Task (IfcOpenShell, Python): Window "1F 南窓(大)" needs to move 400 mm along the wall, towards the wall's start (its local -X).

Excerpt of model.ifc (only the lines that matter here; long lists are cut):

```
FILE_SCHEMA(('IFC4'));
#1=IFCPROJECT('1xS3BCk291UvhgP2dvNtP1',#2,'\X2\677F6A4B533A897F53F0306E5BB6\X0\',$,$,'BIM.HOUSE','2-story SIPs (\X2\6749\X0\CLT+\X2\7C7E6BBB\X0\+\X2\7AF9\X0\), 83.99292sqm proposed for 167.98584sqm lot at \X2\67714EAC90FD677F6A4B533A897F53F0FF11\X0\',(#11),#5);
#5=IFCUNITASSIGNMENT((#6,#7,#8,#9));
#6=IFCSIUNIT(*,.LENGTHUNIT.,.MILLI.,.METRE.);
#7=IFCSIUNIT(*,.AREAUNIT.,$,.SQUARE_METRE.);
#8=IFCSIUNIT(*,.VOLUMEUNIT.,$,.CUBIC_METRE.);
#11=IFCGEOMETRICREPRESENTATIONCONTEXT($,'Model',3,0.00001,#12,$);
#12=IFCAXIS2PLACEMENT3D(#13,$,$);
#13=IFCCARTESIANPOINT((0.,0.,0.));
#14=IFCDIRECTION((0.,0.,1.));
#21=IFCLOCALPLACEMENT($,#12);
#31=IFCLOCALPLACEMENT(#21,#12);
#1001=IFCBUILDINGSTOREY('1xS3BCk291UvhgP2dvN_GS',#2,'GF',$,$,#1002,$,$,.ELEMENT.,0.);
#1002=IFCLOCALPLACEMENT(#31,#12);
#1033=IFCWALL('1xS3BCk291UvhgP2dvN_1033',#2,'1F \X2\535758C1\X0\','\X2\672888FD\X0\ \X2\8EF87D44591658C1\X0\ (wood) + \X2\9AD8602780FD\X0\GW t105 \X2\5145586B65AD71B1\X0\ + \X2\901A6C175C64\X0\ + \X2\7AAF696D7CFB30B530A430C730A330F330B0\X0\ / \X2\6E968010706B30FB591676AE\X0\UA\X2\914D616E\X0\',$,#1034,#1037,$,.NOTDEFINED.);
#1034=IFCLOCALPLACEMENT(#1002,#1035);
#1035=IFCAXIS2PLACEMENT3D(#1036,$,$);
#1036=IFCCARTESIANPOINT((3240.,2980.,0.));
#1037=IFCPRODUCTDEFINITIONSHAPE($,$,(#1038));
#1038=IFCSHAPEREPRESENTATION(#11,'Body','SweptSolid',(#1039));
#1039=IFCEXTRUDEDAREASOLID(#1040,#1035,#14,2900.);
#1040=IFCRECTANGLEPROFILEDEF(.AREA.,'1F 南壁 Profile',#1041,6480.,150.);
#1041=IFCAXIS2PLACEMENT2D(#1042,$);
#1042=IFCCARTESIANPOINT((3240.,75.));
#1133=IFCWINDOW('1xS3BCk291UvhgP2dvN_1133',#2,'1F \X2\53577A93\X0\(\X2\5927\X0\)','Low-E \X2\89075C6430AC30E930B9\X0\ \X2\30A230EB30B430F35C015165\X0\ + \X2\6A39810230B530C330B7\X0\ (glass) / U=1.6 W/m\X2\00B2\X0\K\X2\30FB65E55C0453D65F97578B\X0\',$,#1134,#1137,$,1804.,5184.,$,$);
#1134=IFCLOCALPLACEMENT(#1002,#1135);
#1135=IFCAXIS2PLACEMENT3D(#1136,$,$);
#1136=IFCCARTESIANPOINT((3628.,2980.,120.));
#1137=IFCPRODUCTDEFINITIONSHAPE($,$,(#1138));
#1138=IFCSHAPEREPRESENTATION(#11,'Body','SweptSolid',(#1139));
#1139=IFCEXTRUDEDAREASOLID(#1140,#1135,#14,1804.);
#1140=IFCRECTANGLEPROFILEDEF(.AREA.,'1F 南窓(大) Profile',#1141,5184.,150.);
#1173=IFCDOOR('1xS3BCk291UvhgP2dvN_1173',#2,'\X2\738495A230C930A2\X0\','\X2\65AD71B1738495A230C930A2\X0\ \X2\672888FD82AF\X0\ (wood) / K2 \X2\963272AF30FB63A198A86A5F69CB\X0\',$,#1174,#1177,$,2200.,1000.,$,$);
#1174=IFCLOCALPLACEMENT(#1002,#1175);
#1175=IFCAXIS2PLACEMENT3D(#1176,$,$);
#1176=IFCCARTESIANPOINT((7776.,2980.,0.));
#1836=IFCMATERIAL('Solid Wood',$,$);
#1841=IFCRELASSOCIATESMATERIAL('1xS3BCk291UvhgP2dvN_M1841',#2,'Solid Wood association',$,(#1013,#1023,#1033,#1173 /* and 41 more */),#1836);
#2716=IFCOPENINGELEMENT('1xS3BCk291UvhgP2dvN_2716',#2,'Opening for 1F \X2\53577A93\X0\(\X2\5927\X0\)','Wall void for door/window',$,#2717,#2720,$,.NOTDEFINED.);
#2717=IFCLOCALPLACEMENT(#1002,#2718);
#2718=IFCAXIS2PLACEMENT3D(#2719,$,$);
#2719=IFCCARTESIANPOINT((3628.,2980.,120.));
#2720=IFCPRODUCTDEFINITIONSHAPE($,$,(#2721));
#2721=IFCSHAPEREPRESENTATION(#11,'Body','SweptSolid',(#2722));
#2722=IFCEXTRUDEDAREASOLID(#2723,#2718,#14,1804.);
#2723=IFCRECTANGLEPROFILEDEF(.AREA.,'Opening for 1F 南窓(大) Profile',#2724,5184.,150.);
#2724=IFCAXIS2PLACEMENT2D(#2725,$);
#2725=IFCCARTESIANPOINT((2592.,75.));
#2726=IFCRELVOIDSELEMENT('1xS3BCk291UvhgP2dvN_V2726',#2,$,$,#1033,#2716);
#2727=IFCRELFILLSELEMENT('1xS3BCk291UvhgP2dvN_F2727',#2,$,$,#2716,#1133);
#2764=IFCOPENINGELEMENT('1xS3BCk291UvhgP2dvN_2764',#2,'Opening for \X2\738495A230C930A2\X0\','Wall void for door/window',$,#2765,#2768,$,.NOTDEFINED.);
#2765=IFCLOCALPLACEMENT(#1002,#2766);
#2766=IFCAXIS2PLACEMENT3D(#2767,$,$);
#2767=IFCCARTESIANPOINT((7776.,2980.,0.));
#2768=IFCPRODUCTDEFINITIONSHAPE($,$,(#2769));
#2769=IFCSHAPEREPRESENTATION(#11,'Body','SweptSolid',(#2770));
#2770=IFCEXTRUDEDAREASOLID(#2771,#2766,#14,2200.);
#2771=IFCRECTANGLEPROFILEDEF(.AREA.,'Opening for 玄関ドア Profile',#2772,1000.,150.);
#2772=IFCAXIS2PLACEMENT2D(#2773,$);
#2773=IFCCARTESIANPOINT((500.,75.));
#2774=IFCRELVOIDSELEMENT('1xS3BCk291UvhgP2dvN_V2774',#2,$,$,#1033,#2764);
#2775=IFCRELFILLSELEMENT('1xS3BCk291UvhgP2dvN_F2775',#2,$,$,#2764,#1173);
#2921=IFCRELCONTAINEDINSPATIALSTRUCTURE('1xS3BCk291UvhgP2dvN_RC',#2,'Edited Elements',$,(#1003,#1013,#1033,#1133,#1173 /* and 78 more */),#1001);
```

```python
import ifcopenshell
import ifcopenshell.api.geometry
import ifcopenshell.util.placement
import ifcopenshell.util.unit

model = ifcopenshell.open("model.ifc")
unit_scale = ifcopenshell.util.unit.calculate_unit_scale(model)

window = model.by_id(1133)
opening = window.FillsVoids[0].RelatingOpeningElement
wall = opening.VoidsElements[0].RelatingBuildingElement

wall_matrix = ifcopenshell.util.placement.get_local_placement(wall.ObjectPlacement)
shift = wall_matrix[:3, 0] * -0.4 / unit_scale
before = ifcopenshell.util.placement.get_local_placement(window.ObjectPlacement)[:3, 3].copy()

# The window is not placed relative to its opening, so move both.
for product in (opening, window):
    matrix = ifcopenshell.util.placement.get_local_placement(product.ObjectPlacement)
    matrix[:3, 3] += shift
    ifcopenshell.api.geometry.edit_object_placement(model, product=product, matrix=matrix, is_si=False)

after = ifcopenshell.util.placement.get_local_placement(window.ObjectPlacement)[:3, 3]
print("window moved by", (after - before).round(3) + 0.0)

model.write("model-out.ifc")
```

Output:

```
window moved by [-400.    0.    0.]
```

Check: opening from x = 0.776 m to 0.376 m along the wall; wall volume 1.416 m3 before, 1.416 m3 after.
